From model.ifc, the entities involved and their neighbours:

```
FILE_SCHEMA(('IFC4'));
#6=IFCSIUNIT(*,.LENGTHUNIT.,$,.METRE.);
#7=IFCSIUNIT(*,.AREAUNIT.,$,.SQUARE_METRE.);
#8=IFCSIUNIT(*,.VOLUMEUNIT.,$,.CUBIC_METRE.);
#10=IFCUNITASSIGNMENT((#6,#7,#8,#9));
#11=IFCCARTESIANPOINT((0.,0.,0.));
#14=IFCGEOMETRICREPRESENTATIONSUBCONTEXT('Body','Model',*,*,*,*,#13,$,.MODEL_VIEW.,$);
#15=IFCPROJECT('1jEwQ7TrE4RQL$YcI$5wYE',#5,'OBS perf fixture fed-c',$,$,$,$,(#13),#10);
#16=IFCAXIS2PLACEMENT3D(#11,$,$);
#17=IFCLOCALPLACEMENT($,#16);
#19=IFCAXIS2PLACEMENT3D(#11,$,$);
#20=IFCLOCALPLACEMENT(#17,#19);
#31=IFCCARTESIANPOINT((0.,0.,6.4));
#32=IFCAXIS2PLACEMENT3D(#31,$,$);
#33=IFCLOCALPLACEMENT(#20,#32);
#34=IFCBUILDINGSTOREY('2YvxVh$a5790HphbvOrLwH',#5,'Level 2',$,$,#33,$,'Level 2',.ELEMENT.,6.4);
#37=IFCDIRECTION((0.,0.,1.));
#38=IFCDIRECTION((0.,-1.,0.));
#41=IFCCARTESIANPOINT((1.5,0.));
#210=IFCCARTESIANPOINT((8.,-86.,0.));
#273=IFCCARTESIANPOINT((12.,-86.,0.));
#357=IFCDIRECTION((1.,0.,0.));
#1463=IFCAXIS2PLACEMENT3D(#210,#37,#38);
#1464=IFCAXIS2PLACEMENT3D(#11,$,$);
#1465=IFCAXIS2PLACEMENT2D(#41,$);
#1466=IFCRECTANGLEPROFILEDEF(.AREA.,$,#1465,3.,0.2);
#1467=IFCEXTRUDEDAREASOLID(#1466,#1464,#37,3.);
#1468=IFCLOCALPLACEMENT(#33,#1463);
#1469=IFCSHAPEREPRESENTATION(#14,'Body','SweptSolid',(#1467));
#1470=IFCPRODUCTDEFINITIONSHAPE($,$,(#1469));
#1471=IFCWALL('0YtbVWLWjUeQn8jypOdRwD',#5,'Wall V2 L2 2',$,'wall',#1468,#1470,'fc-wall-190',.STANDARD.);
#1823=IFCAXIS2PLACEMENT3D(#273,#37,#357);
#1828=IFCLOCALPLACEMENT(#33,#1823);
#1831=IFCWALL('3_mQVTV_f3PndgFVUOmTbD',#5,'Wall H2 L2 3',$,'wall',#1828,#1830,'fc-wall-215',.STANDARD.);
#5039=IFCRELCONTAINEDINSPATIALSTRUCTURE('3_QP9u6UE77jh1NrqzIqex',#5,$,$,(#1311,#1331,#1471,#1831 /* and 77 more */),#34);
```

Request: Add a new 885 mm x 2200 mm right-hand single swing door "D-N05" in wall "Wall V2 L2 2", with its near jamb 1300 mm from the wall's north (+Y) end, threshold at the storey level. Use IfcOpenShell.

```python
import numpy as np
import ifcopenshell
import ifcopenshell.api.feature
import ifcopenshell.api.geometry
import ifcopenshell.api.root
import ifcopenshell.api.spatial
import ifcopenshell.geom
import ifcopenshell.util.element
import ifcopenshell.util.placement
import ifcopenshell.util.representation
import ifcopenshell.util.shape
import ifcopenshell.util.unit

model = ifcopenshell.open("model.ifc")
unit_scale = ifcopenshell.util.unit.calculate_unit_scale(model)
settings = ifcopenshell.geom.settings()


def volume(element):
    """Net volume in cubic metres, openings subtracted."""
    shape = ifcopenshell.geom.create_shape(settings, element)
    return ifcopenshell.util.shape.get_volume(shape.geometry)


wall = model.by_guid("0YtbVWLWjUeQn8jypOdRwD")
storey = ifcopenshell.util.element.get_container(wall, ifc_class="IfcBuildingStorey")
context = ifcopenshell.util.representation.get_context(model, "Model", "Body", "MODEL_VIEW")
before = volume(wall)

width, height, from_end, sill = 0.885, 2.2, 1.3, 0.0  # metres

# The wall runs along its own X axis, and the end named is its -X end.
wall_shape = ifcopenshell.geom.create_shape(settings, wall)
x, y, z = ifcopenshell.util.shape.get_vertices(wall_shape.geometry).T
start = x.min() + from_end
face, thickness = float(y.min()), float(y.max() - y.min())
wall_matrix = ifcopenshell.util.placement.get_local_placement(wall.ObjectPlacement)
level = ifcopenshell.util.placement.get_local_placement(storey.ObjectPlacement)[2, 3]


def in_wall(x, y):
    """Placement at x, y metres in the wall's axes, at sill height."""
    matrix = wall_matrix.copy()
    matrix[:, 3] = wall_matrix @ np.array([x / unit_scale, y / unit_scale, 0.0, 1.0])
    matrix[2, 3] = level + sill / unit_scale
    return matrix


# Opening: a box that overshoots both wall faces by 50 mm.
opening = ifcopenshell.api.root.create_entity(model, ifc_class="IfcOpeningElement", predefined_type="OPENING")
box = ifcopenshell.api.geometry.add_wall_representation(
    model, context=context, length=width, height=height, thickness=thickness + 0.1
)
ifcopenshell.api.geometry.assign_representation(model, product=opening, representation=box)
ifcopenshell.api.geometry.edit_object_placement(model, product=opening, matrix=in_wall(start, face - 0.05), is_si=False)
ifcopenshell.api.feature.add_feature(model, feature=opening, element=wall)

door = ifcopenshell.api.root.create_entity(model, ifc_class="IfcDoor", name="D-N05", predefined_type="DOOR")
door.OverallWidth, door.OverallHeight = width / unit_scale, height / unit_scale
door.OperationType = "SINGLE_SWING_RIGHT"
body = ifcopenshell.api.geometry.add_door_representation(
    model,
    context=context,
    overall_width=door.OverallWidth,
    overall_height=door.OverallHeight,
    operation_type="SINGLE_SWING_RIGHT",
    lining_properties={"LiningDepth": thickness / unit_scale, "ThresholdDepth": thickness / unit_scale},
)
ifcopenshell.api.geometry.assign_representation(model, product=door, representation=body)
ifcopenshell.api.spatial.assign_container(model, products=[door], relating_structure=storey)
ifcopenshell.api.feature.add_filling(model, opening=opening, element=door)

# The lining spans the wall, so the door starts at the wall face.
ifcopenshell.api.geometry.edit_object_placement(model, product=door, matrix=in_wall(start, face), is_si=False)

after = volume(wall)

print(f"wall volume {before:.3f} -> {after:.3f} m3")

model.write("model-out.ifc")
```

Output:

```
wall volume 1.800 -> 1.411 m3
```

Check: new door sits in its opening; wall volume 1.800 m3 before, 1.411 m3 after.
